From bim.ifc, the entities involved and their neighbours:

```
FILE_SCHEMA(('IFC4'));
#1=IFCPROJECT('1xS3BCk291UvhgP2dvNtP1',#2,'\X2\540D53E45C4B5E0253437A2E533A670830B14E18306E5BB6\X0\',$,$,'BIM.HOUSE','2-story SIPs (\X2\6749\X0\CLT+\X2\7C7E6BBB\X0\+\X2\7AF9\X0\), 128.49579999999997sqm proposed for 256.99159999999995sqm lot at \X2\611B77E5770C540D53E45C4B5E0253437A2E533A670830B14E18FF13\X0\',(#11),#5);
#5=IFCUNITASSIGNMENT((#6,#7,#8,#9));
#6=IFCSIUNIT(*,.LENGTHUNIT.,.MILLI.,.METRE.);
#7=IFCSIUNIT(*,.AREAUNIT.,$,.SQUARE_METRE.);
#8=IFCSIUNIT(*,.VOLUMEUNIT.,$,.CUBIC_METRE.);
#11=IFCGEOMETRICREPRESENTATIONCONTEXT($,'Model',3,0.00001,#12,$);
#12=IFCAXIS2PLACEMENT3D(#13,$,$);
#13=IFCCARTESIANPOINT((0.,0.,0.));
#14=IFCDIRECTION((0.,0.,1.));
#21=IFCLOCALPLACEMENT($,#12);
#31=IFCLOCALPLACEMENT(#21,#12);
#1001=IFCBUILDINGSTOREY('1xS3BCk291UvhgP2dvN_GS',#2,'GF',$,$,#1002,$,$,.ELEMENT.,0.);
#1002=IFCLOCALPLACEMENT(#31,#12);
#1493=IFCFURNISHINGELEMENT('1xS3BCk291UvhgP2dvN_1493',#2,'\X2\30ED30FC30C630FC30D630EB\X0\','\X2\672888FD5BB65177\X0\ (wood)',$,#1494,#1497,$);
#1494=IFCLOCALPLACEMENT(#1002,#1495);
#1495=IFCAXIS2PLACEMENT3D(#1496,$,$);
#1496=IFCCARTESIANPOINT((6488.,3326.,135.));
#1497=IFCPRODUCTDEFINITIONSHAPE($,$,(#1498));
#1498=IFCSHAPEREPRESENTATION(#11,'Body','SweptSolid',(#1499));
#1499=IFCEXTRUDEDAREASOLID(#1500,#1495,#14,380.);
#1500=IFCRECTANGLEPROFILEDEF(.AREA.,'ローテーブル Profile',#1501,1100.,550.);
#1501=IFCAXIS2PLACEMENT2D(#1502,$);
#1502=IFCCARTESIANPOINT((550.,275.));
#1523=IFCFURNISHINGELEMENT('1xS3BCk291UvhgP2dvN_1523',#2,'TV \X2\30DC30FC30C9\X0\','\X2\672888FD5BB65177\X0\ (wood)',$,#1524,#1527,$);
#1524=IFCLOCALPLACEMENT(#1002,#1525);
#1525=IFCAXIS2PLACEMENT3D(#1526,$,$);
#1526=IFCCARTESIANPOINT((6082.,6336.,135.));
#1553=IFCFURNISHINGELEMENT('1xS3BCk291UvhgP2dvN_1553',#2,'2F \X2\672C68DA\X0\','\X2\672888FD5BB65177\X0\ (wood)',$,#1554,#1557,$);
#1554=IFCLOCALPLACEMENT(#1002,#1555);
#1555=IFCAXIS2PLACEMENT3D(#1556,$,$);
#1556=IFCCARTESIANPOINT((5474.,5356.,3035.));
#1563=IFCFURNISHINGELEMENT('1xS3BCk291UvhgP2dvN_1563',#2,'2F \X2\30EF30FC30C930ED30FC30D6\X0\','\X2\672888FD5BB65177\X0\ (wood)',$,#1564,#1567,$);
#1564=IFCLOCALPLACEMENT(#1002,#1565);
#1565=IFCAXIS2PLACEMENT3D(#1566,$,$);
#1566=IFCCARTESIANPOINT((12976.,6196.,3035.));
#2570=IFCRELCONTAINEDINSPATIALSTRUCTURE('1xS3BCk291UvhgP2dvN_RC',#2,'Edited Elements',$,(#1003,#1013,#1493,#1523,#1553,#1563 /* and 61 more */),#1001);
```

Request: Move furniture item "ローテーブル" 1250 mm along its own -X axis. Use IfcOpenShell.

```python
import ifcopenshell
import ifcopenshell.api.geometry
import ifcopenshell.util.placement

model = ifcopenshell.open("bim.ifc")

item = model.by_guid("1xS3BCk291UvhgP2dvN_1493")
matrix = ifcopenshell.util.placement.get_local_placement(item.ObjectPlacement)
matrix[:3, 3] -= matrix[:3, 0] * 1250.0
ifcopenshell.api.geometry.edit_object_placement(model, product=item, matrix=matrix, is_si=False)

print(ifcopenshell.util.placement.get_local_placement(item.ObjectPlacement).round(3) + 0.0)

model.write("bim_v2.ifc")
```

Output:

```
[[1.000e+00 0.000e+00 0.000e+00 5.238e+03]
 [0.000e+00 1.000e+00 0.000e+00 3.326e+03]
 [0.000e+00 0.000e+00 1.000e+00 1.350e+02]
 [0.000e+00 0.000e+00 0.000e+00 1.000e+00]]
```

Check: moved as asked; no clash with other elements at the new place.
